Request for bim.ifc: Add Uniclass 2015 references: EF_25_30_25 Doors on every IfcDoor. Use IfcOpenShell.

First a look at what the model holds.

```python
import ifcopenshell

model = ifcopenshell.open("bim.ifc")
print(model.schema)
print("classifications:", [c.Name for c in model.by_type("IfcClassification")])
for ifc_class in ("IfcDoor", "IfcRoof", "IfcStair", "IfcWall", "IfcWindow"):
    print(ifc_class, len(model.by_type(ifc_class)))
```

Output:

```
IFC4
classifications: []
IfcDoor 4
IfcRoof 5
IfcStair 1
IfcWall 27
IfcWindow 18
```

```python
import ifcopenshell
import ifcopenshell.api.classification

model = ifcopenshell.open("bim.ifc")

system = ifcopenshell.api.classification.add_classification(model, classification="Uniclass 2015")

codes = {
    "IfcDoor": ("EF_25_30_25", "Doors"),
}
for ifc_class, (code, name) in codes.items():
    products = model.by_type(ifc_class)
    ifcopenshell.api.classification.add_reference(
        model, products=products, classification=system, identification=code, name=name
    )
    print(code, len(products))

model.write("bim_edited.ifc")
```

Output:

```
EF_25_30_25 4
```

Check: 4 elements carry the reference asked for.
